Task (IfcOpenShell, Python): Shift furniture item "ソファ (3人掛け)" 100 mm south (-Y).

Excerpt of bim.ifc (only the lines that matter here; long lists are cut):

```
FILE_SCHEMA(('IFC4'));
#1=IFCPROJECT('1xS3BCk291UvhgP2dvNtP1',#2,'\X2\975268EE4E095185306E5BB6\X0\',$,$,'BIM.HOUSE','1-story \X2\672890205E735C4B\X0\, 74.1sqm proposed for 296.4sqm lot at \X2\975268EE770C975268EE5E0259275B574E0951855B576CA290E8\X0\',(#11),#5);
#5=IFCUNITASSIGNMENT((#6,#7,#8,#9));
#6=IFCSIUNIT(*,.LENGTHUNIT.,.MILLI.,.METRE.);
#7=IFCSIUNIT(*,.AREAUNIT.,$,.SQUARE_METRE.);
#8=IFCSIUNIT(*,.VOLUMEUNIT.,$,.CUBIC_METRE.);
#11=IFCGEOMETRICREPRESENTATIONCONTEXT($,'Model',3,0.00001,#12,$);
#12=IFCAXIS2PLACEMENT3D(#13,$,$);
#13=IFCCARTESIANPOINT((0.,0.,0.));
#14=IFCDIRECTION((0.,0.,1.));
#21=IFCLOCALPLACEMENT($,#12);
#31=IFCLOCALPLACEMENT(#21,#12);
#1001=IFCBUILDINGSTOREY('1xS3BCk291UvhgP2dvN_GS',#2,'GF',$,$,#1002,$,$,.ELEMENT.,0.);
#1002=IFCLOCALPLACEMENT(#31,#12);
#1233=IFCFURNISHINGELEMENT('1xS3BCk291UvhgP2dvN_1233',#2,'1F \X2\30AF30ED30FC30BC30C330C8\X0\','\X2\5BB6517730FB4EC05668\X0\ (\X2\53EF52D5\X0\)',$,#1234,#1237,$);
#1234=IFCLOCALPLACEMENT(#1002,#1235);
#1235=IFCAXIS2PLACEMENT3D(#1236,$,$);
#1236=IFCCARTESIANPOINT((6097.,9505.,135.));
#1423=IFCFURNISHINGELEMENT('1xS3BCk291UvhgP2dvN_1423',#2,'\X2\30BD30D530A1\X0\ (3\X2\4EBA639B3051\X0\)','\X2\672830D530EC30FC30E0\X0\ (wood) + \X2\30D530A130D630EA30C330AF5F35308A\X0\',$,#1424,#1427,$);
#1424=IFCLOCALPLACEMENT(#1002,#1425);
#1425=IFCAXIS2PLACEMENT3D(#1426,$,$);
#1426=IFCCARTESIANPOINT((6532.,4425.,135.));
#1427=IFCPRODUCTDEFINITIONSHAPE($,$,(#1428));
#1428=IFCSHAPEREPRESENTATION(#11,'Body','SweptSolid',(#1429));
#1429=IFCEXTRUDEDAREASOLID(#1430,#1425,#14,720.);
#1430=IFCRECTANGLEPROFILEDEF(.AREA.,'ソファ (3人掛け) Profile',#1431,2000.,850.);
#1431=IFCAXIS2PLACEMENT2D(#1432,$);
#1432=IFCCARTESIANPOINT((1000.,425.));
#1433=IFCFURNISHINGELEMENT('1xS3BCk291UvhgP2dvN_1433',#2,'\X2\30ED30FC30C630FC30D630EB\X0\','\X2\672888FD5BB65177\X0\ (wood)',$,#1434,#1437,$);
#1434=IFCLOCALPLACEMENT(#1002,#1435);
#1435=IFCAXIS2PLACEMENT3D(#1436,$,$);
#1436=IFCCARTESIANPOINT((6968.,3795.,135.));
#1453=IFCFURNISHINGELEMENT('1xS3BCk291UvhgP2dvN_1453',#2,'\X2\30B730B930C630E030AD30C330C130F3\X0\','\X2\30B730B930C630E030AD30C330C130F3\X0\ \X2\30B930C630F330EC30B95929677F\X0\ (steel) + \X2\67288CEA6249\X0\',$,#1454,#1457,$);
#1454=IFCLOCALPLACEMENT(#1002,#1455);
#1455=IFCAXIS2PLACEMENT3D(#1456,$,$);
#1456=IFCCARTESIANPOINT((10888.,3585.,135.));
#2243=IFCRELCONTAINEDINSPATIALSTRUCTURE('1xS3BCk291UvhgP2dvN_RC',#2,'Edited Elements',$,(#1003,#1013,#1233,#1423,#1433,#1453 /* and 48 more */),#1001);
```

```python
import ifcopenshell
import ifcopenshell.api.geometry
import ifcopenshell.util.placement
import ifcopenshell.util.unit

model = ifcopenshell.open("bim.ifc")
unit_scale = ifcopenshell.util.unit.calculate_unit_scale(model)

item = model.by_id(1423)
matrix = ifcopenshell.util.placement.get_local_placement(item.ObjectPlacement)
matrix[1, 3] -= 0.1 / unit_scale
ifcopenshell.api.geometry.edit_object_placement(model, product=item, matrix=matrix, is_si=False)

print(ifcopenshell.util.placement.get_local_placement(item.ObjectPlacement).round(3) + 0.0)

model.write("bim_v2.ifc")
```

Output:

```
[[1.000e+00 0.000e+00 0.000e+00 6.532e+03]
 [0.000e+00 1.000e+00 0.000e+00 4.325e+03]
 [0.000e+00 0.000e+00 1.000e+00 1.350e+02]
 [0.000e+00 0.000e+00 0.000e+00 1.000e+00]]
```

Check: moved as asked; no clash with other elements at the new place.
